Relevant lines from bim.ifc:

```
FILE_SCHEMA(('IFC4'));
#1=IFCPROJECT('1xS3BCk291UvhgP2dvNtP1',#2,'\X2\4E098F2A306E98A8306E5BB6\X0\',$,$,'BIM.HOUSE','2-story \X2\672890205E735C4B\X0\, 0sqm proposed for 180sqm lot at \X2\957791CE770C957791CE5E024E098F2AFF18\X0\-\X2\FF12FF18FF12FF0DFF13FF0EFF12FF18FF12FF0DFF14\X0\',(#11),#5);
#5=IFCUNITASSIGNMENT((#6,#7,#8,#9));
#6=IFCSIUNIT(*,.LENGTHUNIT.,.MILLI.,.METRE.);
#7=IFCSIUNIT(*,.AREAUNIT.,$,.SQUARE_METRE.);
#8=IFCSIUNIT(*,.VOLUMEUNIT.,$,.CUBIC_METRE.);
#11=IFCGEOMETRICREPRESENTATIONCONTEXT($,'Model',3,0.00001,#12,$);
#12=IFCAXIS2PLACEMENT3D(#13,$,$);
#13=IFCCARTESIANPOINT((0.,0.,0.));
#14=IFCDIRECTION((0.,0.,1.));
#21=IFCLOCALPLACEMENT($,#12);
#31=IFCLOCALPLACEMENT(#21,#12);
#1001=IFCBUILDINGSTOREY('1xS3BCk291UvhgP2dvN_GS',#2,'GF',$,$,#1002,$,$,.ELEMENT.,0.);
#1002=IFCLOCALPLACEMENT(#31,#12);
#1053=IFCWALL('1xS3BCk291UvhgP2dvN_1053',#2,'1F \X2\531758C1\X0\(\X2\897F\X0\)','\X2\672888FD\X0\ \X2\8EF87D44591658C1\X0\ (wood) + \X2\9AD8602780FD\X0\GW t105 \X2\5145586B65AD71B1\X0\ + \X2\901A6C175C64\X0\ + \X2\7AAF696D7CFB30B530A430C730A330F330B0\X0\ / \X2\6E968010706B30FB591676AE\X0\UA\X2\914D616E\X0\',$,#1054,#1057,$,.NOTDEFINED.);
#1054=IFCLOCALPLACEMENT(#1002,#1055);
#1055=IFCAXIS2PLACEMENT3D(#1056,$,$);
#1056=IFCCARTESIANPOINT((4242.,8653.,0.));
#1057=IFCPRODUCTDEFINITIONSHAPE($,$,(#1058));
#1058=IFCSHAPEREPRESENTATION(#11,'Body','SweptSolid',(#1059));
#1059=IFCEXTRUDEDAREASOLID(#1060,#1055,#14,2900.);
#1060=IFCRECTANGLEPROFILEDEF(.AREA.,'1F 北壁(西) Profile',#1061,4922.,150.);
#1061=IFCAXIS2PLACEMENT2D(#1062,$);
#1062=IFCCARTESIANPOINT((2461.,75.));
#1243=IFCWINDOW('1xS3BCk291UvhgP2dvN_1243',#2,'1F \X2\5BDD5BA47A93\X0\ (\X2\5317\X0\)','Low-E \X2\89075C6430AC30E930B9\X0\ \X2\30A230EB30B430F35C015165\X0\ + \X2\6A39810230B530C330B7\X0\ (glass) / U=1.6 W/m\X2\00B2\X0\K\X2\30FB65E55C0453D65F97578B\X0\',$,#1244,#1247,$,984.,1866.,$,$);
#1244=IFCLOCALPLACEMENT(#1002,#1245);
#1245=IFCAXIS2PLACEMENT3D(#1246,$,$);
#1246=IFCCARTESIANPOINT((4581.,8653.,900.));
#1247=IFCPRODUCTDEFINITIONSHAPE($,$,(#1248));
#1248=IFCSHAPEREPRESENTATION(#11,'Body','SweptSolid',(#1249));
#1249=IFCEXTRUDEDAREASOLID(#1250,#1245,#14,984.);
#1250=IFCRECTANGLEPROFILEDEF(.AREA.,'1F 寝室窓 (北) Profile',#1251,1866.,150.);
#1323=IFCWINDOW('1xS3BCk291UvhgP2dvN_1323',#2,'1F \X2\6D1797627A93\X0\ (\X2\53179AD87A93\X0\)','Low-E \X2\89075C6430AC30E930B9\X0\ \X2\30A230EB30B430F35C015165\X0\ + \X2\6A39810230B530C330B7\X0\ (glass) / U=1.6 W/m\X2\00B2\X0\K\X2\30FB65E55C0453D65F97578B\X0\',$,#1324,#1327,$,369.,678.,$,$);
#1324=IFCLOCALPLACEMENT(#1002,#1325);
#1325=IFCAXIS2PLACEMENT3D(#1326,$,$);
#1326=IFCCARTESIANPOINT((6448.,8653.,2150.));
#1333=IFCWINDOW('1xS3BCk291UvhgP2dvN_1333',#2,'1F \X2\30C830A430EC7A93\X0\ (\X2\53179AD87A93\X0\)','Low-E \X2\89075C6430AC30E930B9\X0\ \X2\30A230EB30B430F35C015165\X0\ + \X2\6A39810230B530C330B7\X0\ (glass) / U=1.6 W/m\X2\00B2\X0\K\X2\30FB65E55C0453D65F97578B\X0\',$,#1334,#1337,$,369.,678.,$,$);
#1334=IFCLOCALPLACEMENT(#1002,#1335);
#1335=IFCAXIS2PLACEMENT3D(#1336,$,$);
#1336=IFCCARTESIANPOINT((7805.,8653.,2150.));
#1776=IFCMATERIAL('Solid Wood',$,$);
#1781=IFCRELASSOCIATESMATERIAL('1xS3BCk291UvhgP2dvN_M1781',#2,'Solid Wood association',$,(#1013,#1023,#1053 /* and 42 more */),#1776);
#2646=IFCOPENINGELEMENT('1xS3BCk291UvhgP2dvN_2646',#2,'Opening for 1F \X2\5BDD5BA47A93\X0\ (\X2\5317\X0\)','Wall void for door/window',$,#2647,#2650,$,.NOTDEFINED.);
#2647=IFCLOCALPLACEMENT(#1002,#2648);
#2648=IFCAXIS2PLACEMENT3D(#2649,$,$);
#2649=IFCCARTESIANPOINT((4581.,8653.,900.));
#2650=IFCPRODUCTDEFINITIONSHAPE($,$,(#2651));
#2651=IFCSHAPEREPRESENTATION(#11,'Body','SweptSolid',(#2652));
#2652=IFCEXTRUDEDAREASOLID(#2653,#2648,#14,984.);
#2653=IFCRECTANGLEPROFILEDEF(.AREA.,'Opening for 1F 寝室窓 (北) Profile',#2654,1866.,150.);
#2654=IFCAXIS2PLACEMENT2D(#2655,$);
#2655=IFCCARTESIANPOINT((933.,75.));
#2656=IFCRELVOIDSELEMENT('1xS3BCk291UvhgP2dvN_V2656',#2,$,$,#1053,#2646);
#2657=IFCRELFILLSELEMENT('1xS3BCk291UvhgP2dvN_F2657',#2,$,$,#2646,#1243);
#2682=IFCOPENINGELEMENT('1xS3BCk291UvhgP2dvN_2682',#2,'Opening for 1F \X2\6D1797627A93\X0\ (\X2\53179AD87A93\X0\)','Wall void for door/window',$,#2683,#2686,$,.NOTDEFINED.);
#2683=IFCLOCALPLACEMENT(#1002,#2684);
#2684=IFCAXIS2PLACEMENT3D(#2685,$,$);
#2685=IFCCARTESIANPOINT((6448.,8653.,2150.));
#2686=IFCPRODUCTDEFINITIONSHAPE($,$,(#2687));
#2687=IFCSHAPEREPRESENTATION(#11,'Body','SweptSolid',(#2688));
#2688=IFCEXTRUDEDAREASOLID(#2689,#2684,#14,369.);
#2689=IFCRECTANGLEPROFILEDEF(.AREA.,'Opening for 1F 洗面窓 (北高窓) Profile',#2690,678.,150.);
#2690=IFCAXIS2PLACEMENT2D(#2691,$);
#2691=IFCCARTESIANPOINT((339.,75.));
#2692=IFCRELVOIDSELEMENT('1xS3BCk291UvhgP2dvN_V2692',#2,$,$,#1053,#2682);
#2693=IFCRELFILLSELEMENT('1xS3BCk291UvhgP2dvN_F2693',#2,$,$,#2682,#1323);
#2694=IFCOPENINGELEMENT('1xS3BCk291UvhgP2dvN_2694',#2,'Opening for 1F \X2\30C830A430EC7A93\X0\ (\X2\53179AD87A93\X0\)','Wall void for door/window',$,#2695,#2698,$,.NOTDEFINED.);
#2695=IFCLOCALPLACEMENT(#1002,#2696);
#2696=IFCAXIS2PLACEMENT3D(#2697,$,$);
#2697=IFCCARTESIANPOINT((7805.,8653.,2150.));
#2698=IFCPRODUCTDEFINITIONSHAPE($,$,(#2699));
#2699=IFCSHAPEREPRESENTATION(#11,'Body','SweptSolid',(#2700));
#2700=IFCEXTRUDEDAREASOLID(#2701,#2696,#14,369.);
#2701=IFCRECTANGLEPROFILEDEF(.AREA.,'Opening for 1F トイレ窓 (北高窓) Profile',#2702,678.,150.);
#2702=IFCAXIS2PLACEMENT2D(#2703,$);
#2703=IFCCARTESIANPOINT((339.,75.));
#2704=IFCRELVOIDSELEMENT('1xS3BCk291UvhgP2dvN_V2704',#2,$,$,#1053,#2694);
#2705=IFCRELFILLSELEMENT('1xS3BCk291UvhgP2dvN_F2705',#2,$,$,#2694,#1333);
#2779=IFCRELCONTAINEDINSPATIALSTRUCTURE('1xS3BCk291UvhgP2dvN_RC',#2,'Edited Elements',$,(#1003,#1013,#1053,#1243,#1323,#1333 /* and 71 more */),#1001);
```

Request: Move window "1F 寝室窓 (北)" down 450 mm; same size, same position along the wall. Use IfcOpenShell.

```python
import numpy as np
import ifcopenshell
import ifcopenshell.api.geometry
import ifcopenshell.util.placement
import ifcopenshell.util.unit

model = ifcopenshell.open("bim.ifc")
unit_scale = ifcopenshell.util.unit.calculate_unit_scale(model)

window = model.by_guid("1xS3BCk291UvhgP2dvN_1243")
opening = window.FillsVoids[0].RelatingOpeningElement
dz = -0.45 / unit_scale

shift = np.array([0.0, 0.0, dz])
# The window is not placed relative to its opening, so move both.
for product in (opening, window):
    matrix = ifcopenshell.util.placement.get_local_placement(product.ObjectPlacement)
    matrix[:3, 3] += shift
    ifcopenshell.api.geometry.edit_object_placement(model, product=product, matrix=matrix, is_si=False)

print(f"moved by {dz * unit_scale:+.3f} m")

model.write("bim_edited.ifc")
```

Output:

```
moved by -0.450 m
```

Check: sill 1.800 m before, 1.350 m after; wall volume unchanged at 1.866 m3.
